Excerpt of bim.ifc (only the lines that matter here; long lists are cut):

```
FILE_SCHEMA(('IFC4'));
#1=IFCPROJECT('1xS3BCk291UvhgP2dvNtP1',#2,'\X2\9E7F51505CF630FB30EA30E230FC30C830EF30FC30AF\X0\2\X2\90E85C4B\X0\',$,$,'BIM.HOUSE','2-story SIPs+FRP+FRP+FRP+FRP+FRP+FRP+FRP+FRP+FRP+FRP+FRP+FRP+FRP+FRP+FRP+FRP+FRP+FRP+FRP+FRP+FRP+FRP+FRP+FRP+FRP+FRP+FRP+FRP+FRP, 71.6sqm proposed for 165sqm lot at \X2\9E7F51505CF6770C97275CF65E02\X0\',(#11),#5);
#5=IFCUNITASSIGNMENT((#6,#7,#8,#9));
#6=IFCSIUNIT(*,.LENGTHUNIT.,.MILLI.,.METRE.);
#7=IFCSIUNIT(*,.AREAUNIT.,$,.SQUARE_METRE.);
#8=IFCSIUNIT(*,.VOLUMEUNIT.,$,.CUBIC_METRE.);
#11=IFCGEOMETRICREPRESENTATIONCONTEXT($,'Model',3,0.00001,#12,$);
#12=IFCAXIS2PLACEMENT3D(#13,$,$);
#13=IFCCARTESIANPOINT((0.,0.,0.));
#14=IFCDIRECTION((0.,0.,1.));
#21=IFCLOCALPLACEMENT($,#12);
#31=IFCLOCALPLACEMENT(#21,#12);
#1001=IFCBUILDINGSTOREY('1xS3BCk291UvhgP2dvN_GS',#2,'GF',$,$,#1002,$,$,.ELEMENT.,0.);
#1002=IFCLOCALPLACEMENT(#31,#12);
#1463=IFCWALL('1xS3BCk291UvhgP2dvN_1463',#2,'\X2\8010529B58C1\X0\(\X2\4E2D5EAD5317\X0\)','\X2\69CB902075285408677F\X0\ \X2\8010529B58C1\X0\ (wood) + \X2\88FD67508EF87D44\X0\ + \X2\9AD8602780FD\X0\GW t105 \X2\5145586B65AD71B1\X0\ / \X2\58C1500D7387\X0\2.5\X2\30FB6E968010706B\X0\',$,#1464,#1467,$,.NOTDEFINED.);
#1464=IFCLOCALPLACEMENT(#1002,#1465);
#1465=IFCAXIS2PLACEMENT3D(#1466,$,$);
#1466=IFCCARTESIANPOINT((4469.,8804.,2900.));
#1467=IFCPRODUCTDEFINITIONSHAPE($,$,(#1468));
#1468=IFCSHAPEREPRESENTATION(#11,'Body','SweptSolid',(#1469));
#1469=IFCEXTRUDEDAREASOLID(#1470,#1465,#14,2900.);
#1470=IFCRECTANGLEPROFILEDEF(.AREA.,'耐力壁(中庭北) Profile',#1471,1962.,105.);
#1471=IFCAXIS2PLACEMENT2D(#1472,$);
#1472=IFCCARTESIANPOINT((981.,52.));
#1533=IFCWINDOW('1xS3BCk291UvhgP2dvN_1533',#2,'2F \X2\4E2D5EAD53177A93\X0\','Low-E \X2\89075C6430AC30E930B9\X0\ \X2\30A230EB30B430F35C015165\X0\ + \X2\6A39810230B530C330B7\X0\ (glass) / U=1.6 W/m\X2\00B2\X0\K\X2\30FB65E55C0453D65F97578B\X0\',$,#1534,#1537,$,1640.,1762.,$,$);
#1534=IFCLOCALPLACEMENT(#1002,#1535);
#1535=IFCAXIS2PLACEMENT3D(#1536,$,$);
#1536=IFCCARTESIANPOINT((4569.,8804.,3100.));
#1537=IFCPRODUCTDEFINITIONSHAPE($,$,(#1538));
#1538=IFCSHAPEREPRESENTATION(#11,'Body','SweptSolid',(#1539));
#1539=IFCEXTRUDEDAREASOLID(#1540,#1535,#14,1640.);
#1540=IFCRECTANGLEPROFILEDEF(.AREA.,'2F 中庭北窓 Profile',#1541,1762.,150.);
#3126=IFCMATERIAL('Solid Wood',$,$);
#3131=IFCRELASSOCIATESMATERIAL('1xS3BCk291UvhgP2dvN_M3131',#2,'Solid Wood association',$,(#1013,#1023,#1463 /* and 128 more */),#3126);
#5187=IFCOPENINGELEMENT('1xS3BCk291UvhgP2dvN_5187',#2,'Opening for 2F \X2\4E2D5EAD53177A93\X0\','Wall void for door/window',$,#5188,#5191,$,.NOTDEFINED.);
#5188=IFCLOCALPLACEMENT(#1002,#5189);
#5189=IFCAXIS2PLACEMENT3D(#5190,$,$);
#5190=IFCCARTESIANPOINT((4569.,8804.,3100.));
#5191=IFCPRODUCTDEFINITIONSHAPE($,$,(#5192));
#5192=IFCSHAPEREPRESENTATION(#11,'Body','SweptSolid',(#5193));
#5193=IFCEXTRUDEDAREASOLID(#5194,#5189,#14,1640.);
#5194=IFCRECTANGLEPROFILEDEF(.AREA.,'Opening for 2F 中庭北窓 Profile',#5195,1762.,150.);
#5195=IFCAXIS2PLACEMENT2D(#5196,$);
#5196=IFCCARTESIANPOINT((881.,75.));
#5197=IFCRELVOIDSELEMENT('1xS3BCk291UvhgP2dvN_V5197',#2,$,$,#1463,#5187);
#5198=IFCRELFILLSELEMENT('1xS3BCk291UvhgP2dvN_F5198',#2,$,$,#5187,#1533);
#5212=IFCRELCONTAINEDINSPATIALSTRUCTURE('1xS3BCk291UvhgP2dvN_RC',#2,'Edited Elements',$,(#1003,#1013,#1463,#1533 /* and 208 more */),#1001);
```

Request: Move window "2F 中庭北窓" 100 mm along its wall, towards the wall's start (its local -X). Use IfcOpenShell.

```python
import ifcopenshell
import ifcopenshell.api.geometry
import ifcopenshell.util.placement
import ifcopenshell.util.unit

model = ifcopenshell.open("bim.ifc")
unit_scale = ifcopenshell.util.unit.calculate_unit_scale(model)

window = model.by_id(1533)
opening = window.FillsVoids[0].RelatingOpeningElement
wall = opening.VoidsElements[0].RelatingBuildingElement

wall_matrix = ifcopenshell.util.placement.get_local_placement(wall.ObjectPlacement)
shift = wall_matrix[:3, 0] * -0.1 / unit_scale
before = ifcopenshell.util.placement.get_local_placement(window.ObjectPlacement)[:3, 3].copy()

# The window is not placed relative to its opening, so move both.
for product in (opening, window):
    matrix = ifcopenshell.util.placement.get_local_placement(product.ObjectPlacement)
    matrix[:3, 3] += shift
    ifcopenshell.api.geometry.edit_object_placement(model, product=product, matrix=matrix, is_si=False)

after = ifcopenshell.util.placement.get_local_placement(window.ObjectPlacement)[:3, 3]
print("window moved by", (after - before).round(3) + 0.0)

model.write("bim-out.ifc")
```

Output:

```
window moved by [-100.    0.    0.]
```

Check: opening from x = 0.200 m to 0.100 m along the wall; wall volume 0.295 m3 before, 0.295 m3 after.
